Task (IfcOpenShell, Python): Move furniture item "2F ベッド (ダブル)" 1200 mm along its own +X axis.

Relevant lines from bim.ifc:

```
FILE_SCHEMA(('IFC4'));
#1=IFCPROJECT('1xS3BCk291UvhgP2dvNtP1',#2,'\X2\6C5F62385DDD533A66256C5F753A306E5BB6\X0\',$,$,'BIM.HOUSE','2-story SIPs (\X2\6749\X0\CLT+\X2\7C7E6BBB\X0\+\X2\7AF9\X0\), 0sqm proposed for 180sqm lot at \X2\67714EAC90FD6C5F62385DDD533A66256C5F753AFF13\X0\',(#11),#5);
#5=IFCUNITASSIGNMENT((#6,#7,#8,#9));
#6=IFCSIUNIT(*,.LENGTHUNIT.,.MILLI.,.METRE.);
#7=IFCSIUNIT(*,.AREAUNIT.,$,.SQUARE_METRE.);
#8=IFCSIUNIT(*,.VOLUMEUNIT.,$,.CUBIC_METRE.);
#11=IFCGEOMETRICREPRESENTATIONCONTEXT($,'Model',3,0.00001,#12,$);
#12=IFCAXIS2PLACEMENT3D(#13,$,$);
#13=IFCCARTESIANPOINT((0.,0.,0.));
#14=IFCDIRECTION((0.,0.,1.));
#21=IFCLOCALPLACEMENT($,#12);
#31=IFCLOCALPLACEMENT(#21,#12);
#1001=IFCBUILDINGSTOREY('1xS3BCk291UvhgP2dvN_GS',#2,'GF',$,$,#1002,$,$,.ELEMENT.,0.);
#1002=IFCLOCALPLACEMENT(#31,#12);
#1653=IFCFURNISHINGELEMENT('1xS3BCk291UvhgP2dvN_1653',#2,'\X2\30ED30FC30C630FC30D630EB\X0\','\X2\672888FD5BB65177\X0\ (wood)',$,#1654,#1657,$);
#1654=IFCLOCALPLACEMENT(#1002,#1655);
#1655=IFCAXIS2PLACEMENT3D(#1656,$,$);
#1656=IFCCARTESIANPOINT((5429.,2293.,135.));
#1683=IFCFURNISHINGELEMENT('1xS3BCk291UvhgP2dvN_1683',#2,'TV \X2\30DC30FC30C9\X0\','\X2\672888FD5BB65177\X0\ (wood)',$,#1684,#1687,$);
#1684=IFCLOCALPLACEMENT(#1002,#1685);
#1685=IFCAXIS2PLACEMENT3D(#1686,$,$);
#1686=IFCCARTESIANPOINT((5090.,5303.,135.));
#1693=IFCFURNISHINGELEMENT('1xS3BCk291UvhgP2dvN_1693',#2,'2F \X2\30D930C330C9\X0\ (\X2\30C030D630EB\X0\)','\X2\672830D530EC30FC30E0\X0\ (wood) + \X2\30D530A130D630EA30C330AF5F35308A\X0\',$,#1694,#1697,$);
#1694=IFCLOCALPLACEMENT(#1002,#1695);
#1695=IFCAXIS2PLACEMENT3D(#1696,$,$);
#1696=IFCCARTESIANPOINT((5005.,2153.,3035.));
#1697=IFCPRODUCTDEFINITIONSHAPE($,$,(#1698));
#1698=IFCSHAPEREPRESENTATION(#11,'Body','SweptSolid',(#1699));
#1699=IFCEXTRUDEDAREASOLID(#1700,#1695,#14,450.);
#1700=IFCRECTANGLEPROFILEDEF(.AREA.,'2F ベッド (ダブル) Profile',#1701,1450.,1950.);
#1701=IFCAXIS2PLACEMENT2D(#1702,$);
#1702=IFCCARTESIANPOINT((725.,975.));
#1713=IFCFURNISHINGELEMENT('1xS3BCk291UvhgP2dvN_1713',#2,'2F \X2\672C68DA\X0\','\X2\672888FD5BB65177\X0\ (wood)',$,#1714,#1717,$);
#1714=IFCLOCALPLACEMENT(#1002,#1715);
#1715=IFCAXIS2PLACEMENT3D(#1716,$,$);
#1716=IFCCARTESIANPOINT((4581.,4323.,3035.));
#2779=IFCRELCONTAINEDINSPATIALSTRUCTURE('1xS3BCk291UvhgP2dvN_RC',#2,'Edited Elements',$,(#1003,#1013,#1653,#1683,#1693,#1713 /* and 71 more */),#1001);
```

```python
import ifcopenshell
import ifcopenshell.api.geometry
import ifcopenshell.util.placement
import ifcopenshell.util.unit

model = ifcopenshell.open("bim.ifc")
unit_scale = ifcopenshell.util.unit.calculate_unit_scale(model)

item = model.by_id(1693)
matrix = ifcopenshell.util.placement.get_local_placement(item.ObjectPlacement)
matrix[:3, 3] += matrix[:3, 0] * 1.2 / unit_scale
ifcopenshell.api.geometry.edit_object_placement(model, product=item, matrix=matrix, is_si=False)

print(ifcopenshell.util.placement.get_local_placement(item.ObjectPlacement).round(3) + 0.0)

model.write("bim_updated.ifc")
```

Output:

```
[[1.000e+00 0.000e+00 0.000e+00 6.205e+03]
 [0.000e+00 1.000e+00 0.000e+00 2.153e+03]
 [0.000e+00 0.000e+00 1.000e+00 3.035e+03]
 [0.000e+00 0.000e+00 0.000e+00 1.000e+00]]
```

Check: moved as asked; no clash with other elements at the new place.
